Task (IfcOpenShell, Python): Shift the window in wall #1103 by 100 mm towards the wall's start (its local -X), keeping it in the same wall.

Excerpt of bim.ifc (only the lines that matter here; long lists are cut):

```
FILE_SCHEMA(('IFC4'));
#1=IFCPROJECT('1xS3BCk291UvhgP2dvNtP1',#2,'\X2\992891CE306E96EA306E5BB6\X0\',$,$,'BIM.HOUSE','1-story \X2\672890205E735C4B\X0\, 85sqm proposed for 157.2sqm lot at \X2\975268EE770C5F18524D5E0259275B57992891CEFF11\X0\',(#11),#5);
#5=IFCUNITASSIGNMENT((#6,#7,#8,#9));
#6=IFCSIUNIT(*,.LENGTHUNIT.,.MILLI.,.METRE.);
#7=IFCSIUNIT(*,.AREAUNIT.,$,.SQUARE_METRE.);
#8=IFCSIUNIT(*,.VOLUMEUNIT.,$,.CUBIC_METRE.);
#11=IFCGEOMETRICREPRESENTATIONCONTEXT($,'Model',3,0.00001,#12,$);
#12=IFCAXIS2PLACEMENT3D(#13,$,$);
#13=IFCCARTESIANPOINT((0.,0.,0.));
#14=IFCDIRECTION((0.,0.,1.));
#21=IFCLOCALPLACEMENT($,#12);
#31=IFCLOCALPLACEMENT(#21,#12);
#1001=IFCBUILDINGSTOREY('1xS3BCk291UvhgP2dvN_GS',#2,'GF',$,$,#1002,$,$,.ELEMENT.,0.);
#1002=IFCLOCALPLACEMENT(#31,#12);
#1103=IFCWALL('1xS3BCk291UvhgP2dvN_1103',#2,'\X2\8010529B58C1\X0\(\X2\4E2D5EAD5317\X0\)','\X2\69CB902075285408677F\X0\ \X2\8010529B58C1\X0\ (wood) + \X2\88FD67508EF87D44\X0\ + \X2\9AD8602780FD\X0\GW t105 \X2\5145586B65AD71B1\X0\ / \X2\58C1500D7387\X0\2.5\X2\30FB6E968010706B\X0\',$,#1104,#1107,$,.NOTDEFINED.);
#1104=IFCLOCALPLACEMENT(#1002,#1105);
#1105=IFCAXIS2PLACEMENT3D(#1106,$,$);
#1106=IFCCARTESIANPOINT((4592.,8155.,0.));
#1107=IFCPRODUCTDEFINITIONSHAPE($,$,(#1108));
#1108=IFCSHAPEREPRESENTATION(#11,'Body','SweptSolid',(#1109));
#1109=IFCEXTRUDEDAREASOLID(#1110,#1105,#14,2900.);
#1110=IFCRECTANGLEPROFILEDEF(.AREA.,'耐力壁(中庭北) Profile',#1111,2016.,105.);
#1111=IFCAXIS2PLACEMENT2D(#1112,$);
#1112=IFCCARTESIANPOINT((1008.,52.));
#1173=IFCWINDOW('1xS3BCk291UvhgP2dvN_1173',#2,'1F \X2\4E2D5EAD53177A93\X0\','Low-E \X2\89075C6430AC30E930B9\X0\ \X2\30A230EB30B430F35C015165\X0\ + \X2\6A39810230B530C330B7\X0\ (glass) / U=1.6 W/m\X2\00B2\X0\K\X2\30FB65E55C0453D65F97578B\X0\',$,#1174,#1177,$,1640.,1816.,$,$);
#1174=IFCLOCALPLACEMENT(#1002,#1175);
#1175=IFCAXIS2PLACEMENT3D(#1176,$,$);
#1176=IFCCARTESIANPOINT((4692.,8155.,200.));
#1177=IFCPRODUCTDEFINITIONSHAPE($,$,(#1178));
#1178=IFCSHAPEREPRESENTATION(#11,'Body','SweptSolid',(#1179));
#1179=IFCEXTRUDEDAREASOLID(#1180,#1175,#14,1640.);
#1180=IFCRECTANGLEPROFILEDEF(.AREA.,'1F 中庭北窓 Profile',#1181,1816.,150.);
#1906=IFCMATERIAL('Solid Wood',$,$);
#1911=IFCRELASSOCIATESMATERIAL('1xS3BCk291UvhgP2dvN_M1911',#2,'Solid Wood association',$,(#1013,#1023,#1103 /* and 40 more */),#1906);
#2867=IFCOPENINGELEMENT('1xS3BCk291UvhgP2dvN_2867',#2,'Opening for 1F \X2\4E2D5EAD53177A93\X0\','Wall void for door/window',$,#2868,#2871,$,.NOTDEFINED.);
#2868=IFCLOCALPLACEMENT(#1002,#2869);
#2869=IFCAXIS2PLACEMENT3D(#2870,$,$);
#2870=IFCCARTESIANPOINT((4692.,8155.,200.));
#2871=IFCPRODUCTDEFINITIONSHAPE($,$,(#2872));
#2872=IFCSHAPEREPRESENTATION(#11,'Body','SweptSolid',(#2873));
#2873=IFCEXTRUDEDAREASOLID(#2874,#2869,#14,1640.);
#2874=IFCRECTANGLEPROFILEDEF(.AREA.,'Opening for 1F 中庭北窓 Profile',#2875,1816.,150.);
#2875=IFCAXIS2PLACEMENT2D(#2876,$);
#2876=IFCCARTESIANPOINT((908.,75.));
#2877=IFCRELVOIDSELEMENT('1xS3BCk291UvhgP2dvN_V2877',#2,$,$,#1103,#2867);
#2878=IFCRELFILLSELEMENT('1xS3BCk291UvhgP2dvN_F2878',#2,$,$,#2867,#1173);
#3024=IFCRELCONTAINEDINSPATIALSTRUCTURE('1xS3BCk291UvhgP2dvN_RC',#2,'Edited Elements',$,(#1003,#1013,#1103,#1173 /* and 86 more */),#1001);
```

```python
import ifcopenshell
import ifcopenshell.api.geometry
import ifcopenshell.util.placement

model = ifcopenshell.open("bim.ifc")

window = model.by_id(1173)
opening = window.FillsVoids[0].RelatingOpeningElement
wall = opening.VoidsElements[0].RelatingBuildingElement

wall_matrix = ifcopenshell.util.placement.get_local_placement(wall.ObjectPlacement)
shift = wall_matrix[:3, 0] * -100.0
before = ifcopenshell.util.placement.get_local_placement(window.ObjectPlacement)[:3, 3].copy()

# The window is not placed relative to its opening, so move both.
for product in (opening, window):
    matrix = ifcopenshell.util.placement.get_local_placement(product.ObjectPlacement)
    matrix[:3, 3] += shift
    ifcopenshell.api.geometry.edit_object_placement(model, product=product, matrix=matrix, is_si=False)

after = ifcopenshell.util.placement.get_local_placement(window.ObjectPlacement)[:3, 3]
print("window moved by", (after - before).round(3) + 0.0)

model.write("bim_edited.ifc")
```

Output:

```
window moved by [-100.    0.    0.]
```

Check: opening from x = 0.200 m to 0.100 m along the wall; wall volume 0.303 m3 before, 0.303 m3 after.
